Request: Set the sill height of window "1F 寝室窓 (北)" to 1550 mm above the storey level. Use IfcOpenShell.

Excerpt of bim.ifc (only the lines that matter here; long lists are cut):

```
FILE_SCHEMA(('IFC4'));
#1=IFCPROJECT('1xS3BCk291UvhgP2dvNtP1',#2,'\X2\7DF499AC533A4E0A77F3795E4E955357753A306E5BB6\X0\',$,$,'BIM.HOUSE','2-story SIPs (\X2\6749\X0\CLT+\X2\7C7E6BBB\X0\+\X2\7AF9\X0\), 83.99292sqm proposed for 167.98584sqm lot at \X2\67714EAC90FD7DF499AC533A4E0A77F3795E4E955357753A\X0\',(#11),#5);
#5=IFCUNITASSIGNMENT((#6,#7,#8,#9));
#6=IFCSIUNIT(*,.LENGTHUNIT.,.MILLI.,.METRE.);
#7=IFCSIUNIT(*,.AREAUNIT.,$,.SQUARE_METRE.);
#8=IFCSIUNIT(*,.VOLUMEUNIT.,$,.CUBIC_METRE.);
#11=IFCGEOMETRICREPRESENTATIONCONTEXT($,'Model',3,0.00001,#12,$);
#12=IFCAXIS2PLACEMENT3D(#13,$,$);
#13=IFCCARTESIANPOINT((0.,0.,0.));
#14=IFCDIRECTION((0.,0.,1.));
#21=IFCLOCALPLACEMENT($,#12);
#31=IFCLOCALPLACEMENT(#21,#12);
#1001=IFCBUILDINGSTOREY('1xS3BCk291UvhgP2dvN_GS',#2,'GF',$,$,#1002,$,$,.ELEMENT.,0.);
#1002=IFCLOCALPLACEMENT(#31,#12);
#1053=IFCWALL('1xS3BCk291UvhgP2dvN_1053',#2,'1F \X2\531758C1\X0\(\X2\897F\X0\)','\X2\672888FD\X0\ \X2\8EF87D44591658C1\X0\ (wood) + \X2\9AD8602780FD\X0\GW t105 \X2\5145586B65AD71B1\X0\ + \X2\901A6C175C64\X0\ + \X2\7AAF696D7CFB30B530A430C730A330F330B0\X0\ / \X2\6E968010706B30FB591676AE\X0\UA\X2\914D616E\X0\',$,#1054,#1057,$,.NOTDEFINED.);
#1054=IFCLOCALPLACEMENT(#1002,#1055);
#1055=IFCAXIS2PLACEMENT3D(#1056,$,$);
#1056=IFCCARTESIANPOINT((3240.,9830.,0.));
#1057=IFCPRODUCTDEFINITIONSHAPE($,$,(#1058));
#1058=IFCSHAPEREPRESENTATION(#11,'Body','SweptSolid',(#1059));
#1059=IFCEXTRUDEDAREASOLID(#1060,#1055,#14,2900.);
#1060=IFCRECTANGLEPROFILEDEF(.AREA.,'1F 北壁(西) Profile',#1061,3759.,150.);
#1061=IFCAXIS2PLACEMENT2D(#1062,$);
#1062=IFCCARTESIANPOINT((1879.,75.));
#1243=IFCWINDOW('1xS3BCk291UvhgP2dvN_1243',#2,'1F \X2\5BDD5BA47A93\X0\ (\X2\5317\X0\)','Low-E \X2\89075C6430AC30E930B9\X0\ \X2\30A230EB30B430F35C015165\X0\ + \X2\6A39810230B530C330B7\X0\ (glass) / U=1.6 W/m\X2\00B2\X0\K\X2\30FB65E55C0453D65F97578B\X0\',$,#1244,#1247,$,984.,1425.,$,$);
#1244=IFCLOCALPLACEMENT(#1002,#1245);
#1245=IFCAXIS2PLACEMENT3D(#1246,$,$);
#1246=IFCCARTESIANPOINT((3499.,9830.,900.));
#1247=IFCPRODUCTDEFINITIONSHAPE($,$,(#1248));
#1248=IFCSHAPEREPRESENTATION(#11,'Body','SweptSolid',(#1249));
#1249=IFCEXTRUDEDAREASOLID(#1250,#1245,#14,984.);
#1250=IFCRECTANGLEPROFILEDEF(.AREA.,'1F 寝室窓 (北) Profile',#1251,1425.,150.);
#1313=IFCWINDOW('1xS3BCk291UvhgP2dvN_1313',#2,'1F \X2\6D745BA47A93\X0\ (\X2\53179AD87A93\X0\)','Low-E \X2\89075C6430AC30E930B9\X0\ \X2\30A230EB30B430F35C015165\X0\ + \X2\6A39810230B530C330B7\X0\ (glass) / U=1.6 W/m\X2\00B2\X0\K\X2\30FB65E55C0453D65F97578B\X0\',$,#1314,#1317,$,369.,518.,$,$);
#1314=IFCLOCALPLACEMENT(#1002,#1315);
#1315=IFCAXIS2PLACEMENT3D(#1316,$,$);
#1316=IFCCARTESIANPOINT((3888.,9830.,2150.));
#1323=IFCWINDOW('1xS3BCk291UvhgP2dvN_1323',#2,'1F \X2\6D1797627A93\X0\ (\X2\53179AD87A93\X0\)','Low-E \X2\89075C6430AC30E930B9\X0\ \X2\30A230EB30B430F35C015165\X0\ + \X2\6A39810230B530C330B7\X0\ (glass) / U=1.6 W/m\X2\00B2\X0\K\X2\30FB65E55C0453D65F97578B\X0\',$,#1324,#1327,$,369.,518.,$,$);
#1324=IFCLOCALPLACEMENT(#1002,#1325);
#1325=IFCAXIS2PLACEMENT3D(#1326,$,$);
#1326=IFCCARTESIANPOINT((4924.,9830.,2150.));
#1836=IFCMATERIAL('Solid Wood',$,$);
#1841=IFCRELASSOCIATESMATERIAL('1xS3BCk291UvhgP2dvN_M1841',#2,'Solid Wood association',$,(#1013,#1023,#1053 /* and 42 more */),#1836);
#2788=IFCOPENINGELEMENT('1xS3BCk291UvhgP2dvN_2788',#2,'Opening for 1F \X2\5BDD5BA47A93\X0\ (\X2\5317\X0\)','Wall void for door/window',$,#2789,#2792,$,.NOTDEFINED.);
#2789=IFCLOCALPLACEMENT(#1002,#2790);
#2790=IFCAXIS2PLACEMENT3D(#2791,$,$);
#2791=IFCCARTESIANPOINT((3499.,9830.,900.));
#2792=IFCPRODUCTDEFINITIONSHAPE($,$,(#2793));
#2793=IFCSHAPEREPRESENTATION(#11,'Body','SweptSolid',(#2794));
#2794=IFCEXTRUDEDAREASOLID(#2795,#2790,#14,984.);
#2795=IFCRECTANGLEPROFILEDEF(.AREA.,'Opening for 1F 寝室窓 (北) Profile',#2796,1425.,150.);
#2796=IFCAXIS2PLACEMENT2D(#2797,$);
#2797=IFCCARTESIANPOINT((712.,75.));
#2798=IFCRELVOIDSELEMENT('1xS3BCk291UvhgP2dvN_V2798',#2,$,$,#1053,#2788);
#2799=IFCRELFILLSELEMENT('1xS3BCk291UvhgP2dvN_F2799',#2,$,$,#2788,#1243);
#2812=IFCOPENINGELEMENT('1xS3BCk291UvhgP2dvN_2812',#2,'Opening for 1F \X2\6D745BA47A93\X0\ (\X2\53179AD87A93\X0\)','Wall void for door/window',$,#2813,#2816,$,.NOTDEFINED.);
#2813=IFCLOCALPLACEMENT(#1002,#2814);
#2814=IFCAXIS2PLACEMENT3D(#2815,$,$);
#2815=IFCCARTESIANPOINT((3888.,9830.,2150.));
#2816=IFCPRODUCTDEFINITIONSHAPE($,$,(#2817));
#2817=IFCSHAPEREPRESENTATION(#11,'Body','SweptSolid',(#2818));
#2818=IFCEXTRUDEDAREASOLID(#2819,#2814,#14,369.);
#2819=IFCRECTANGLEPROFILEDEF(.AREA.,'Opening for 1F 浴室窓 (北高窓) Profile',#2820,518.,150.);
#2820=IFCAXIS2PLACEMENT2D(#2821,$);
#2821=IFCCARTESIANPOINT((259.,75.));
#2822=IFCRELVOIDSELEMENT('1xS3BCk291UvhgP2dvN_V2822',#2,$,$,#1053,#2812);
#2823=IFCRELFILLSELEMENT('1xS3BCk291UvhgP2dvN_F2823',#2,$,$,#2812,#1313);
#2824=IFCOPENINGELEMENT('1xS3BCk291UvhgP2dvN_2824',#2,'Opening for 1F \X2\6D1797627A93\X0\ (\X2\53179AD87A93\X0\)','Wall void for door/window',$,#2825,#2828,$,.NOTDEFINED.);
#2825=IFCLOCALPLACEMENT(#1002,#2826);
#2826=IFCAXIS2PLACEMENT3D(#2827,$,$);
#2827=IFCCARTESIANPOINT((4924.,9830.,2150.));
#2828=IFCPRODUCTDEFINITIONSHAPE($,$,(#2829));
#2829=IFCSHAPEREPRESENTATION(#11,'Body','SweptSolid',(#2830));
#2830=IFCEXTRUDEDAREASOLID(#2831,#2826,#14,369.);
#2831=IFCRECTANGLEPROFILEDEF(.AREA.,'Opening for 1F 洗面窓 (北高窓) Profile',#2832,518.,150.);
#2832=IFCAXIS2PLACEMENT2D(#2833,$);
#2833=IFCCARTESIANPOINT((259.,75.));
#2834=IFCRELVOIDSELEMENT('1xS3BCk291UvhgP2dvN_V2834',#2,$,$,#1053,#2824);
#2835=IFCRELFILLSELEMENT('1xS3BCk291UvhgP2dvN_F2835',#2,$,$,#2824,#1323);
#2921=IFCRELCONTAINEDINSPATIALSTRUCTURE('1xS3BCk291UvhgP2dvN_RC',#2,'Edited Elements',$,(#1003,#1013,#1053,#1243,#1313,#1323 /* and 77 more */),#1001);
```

```python
import numpy as np
import ifcopenshell
import ifcopenshell.api.geometry
import ifcopenshell.geom
import ifcopenshell.util.element
import ifcopenshell.util.placement
import ifcopenshell.util.shape
import ifcopenshell.util.unit

model = ifcopenshell.open("bim.ifc")
unit_scale = ifcopenshell.util.unit.calculate_unit_scale(model)

window = model.by_guid("1xS3BCk291UvhgP2dvN_1243")
opening = window.FillsVoids[0].RelatingOpeningElement
storey = ifcopenshell.util.element.get_container(window, ifc_class="IfcBuildingStorey")
level = ifcopenshell.util.placement.get_local_placement(storey.ObjectPlacement)[2, 3]

# The opening's origin need not be at the sill, so measure its lowest point.
shape = ifcopenshell.geom.create_shape(ifcopenshell.geom.settings(), opening)
bottom = ifcopenshell.util.shape.get_shape_bottom_elevation(shape, shape.geometry) / unit_scale
dz = level + 1.55 / unit_scale - bottom

shift = np.array([0.0, 0.0, dz])
# The window is not placed relative to its opening, so move both.
for product in (opening, window):
    matrix = ifcopenshell.util.placement.get_local_placement(product.ObjectPlacement)
    matrix[:3, 3] += shift
    ifcopenshell.api.geometry.edit_object_placement(model, product=product, matrix=matrix, is_si=False)

print(f"moved by {dz * unit_scale:+.3f} m")

model.write("bim_rev.ifc")
```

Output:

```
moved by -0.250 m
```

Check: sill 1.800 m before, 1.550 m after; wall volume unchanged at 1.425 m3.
